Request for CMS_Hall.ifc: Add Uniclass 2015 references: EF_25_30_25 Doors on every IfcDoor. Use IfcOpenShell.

First a look at what the model holds.

```python
import ifcopenshell

model = ifcopenshell.open("CMS_Hall.ifc")
print(model.schema)
print("classifications:", [c.Name for c in model.by_type("IfcClassification")])
for ifc_class in ("IfcDoor", "IfcRoof", "IfcStair", "IfcWall", "IfcWindow"):
    print(ifc_class, len(model.by_type(ifc_class)))
```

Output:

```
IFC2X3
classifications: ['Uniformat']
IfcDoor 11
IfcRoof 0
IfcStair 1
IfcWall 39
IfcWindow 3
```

```python
import ifcopenshell
import ifcopenshell.api.classification

model = ifcopenshell.open("CMS_Hall.ifc")

# IFC2X3 requires Source and Edition and has no link from the project to the system.
system = model.create_entity("IfcClassification", Source="NBS", Edition="2015", Name="Uniclass 2015")

codes = {
    "IfcDoor": ("EF_25_30_25", "Doors"),
}
for ifc_class, (code, name) in codes.items():
    products = model.by_type(ifc_class)
    ifcopenshell.api.classification.add_reference(
        model, products=products, classification=system, identification=code, name=name
    )
    print(code, len(products))

model.write("CMS_Hall_rev.ifc")
```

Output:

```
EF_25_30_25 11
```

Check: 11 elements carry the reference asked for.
